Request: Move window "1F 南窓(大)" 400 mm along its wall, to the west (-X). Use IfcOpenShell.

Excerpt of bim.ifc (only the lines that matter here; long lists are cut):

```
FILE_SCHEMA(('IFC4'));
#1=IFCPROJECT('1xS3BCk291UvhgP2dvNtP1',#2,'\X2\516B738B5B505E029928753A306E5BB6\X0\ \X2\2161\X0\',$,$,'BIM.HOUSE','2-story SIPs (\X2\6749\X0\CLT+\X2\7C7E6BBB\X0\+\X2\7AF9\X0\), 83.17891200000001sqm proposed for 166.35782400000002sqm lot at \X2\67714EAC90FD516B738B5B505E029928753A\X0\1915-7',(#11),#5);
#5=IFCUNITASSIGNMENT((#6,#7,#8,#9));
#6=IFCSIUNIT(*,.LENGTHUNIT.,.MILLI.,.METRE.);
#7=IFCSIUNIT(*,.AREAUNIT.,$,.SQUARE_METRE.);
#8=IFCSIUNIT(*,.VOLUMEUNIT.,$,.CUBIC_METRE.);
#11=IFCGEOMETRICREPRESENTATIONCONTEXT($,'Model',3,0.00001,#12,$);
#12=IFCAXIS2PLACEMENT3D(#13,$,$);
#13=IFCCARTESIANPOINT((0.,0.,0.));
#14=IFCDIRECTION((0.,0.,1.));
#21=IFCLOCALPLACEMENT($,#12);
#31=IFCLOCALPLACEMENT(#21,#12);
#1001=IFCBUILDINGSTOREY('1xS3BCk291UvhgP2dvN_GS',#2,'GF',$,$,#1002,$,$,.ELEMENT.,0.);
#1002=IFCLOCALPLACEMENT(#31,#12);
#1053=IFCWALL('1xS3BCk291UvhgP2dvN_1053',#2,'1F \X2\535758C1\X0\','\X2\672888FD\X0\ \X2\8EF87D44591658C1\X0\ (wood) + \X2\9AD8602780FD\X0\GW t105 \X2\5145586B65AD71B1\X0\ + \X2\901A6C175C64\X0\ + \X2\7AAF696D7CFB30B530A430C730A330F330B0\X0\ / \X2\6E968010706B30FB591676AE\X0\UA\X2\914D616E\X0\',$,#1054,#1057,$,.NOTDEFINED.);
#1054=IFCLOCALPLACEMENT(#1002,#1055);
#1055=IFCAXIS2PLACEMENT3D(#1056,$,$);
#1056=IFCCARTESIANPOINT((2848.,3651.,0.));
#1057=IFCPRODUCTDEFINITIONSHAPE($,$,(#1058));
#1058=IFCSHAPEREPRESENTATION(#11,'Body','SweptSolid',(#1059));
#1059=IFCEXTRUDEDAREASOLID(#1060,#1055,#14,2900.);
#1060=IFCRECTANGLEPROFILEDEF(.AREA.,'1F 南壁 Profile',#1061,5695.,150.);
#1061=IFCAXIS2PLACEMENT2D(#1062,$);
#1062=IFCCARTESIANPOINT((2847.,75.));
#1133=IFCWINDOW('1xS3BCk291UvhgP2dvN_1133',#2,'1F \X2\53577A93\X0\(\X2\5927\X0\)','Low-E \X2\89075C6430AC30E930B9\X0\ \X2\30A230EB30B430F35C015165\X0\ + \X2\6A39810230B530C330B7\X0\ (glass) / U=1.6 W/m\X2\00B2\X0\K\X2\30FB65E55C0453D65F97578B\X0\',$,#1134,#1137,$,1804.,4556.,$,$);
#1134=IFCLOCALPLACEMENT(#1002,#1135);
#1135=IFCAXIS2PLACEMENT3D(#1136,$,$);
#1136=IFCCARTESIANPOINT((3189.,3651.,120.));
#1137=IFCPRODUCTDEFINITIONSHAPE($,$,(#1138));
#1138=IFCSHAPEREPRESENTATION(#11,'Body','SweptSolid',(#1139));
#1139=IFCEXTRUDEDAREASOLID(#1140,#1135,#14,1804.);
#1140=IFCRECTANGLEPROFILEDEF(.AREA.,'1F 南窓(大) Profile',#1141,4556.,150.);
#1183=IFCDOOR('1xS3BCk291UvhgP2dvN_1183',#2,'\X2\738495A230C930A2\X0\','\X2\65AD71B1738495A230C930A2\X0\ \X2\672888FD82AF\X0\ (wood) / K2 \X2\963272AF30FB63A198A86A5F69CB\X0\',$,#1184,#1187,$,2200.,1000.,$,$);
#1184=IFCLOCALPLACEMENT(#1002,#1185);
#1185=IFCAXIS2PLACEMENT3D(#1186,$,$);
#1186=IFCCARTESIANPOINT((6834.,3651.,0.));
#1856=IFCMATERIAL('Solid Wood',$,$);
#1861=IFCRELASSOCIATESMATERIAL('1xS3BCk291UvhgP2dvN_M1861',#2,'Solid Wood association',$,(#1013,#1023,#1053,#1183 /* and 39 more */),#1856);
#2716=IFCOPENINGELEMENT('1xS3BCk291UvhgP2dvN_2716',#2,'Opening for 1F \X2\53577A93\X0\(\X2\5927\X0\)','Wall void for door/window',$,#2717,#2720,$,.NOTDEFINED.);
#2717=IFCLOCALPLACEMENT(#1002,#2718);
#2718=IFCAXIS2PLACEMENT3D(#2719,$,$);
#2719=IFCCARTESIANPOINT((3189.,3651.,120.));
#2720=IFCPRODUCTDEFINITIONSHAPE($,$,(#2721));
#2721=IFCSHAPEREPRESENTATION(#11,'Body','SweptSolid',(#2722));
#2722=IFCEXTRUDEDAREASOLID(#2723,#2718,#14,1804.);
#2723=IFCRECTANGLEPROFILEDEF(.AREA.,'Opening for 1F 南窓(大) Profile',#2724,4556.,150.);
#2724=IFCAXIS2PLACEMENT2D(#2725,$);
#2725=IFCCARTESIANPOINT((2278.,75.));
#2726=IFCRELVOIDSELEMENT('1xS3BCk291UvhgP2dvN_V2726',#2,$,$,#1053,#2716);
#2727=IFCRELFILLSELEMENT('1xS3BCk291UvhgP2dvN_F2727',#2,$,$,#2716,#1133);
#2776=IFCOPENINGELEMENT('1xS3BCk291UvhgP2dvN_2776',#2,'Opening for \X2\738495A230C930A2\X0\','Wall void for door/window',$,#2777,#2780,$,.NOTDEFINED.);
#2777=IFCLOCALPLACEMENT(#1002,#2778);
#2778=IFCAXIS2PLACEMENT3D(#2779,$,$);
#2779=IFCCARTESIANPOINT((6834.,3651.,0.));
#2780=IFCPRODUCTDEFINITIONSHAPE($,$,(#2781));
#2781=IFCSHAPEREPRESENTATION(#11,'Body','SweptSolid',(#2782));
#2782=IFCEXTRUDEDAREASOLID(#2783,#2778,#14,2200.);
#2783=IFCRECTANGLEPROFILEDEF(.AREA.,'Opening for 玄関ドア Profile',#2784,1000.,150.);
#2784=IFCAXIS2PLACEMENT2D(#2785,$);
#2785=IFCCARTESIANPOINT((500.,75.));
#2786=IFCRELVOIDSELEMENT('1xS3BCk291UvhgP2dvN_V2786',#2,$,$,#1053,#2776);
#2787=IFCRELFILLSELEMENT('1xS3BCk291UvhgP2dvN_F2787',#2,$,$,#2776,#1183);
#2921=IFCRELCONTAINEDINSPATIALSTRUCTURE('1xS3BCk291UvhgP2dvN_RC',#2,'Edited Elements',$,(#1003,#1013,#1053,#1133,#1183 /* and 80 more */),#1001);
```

```python
import ifcopenshell
import ifcopenshell.api.geometry
import ifcopenshell.util.placement
import ifcopenshell.util.unit

model = ifcopenshell.open("bim.ifc")
unit_scale = ifcopenshell.util.unit.calculate_unit_scale(model)

window = model.by_id(1133)
opening = window.FillsVoids[0].RelatingOpeningElement
wall = opening.VoidsElements[0].RelatingBuildingElement

wall_matrix = ifcopenshell.util.placement.get_local_placement(wall.ObjectPlacement)
shift = wall_matrix[:3, 0] * -0.4 / unit_scale
before = ifcopenshell.util.placement.get_local_placement(window.ObjectPlacement)[:3, 3].copy()

# The window is not placed relative to its opening, so move both.
for product in (opening, window):
    matrix = ifcopenshell.util.placement.get_local_placement(product.ObjectPlacement)
    matrix[:3, 3] += shift
    ifcopenshell.api.geometry.edit_object_placement(model, product=product, matrix=matrix, is_si=False)

after = ifcopenshell.util.placement.get_local_placement(window.ObjectPlacement)[:3, 3]
print("window moved by", (after - before).round(3) + 0.0)

model.write("bim_edited.ifc")
```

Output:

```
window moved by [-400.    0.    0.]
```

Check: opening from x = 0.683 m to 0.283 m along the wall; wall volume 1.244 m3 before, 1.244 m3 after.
